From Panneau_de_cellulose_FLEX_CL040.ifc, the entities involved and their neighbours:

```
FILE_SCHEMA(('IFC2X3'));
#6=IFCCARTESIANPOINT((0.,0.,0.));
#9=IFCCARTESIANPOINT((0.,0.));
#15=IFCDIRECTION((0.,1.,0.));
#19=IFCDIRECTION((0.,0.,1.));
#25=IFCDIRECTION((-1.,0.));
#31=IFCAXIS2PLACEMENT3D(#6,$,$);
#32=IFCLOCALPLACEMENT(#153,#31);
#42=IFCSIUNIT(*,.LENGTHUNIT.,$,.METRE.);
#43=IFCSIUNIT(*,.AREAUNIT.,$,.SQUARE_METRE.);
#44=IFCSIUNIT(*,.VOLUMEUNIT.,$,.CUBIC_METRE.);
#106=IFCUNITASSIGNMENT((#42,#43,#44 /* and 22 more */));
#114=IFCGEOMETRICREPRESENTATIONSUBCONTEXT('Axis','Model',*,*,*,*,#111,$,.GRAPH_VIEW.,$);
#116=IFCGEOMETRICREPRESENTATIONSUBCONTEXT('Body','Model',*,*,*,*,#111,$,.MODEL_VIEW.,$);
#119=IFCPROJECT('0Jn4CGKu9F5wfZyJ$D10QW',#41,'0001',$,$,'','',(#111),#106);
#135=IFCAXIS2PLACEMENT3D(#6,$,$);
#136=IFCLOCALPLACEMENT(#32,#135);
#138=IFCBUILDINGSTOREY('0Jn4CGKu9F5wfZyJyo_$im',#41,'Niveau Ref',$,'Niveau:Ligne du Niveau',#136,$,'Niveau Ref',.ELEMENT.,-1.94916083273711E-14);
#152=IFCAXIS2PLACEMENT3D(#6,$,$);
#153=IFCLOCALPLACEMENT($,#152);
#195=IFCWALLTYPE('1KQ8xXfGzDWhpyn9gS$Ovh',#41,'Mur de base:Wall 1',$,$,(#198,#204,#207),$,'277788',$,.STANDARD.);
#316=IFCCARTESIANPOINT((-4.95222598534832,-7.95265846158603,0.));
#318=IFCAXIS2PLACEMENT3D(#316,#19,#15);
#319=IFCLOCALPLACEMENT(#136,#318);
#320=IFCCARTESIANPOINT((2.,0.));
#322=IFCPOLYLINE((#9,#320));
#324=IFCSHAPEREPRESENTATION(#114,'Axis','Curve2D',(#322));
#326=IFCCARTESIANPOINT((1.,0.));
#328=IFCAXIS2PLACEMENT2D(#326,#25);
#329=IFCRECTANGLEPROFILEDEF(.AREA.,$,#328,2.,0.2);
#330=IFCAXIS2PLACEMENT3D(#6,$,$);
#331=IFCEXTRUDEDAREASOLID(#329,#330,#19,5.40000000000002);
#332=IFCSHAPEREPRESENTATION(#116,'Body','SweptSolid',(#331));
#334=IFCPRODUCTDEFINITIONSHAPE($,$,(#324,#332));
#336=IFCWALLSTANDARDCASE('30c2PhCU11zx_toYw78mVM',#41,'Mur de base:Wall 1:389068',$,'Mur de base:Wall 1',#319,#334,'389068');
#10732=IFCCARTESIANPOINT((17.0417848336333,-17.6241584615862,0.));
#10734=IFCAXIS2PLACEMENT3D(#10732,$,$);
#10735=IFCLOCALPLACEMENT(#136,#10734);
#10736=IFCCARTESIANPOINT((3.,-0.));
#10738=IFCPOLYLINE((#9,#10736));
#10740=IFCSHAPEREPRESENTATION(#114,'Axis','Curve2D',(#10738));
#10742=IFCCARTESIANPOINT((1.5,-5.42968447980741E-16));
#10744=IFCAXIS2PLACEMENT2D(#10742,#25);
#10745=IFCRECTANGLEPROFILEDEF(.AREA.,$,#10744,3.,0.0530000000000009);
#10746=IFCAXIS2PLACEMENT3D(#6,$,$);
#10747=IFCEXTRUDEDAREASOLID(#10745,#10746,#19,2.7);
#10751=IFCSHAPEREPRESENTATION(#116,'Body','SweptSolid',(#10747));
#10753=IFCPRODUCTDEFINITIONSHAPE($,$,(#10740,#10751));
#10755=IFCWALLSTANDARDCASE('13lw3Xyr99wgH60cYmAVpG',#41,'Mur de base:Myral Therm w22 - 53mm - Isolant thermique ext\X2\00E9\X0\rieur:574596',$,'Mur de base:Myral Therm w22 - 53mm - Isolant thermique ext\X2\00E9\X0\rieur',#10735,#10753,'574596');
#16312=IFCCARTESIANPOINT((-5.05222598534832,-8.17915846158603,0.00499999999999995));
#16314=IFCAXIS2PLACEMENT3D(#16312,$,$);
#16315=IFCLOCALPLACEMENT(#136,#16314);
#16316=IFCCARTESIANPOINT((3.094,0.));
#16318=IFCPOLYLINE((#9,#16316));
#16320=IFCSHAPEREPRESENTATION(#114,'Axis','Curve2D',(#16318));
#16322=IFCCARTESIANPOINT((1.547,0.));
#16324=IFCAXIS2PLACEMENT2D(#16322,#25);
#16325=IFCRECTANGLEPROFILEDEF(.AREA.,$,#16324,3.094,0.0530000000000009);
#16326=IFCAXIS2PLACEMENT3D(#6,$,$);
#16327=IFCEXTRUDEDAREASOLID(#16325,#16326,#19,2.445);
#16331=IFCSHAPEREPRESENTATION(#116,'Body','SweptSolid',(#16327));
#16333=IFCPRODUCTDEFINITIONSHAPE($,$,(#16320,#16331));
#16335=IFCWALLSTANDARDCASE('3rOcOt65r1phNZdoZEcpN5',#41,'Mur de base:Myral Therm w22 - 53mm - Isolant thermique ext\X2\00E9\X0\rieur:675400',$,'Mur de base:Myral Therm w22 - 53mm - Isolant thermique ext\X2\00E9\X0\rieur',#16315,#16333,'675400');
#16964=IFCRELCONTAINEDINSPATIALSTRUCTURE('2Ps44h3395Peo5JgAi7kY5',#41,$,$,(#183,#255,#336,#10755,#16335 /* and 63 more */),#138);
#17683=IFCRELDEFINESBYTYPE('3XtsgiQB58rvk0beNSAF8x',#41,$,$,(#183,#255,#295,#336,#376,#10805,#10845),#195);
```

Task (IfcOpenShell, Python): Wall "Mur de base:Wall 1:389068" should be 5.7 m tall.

```python
import ifcopenshell
import ifcopenshell.geom
import ifcopenshell.util.representation
import ifcopenshell.util.shape

model = ifcopenshell.open("Panneau_de_cellulose_FLEX_CL040.ifc")
settings = ifcopenshell.geom.settings()


def volume(element):
    """Net volume in cubic metres, openings subtracted."""
    shape = ifcopenshell.geom.create_shape(settings, element)
    return ifcopenshell.util.shape.get_volume(shape.geometry)


wall = model.by_guid("30c2PhCU11zx_toYw78mVM")
before = volume(wall)

body = ifcopenshell.util.representation.get_representation(wall, "Model", "Body")
solid = body.Items[0]
old_height = solid.Depth
solid.Depth = 5.7
after = volume(wall)

print(f"height {old_height:g} -> {solid.Depth:g}, volume {before:.3f} -> {after:.3f} m3")

model.write("Panneau_de_cellulose_FLEX_CL040-out.ifc")
```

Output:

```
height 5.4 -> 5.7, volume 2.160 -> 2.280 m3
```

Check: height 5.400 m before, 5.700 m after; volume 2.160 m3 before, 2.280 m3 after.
